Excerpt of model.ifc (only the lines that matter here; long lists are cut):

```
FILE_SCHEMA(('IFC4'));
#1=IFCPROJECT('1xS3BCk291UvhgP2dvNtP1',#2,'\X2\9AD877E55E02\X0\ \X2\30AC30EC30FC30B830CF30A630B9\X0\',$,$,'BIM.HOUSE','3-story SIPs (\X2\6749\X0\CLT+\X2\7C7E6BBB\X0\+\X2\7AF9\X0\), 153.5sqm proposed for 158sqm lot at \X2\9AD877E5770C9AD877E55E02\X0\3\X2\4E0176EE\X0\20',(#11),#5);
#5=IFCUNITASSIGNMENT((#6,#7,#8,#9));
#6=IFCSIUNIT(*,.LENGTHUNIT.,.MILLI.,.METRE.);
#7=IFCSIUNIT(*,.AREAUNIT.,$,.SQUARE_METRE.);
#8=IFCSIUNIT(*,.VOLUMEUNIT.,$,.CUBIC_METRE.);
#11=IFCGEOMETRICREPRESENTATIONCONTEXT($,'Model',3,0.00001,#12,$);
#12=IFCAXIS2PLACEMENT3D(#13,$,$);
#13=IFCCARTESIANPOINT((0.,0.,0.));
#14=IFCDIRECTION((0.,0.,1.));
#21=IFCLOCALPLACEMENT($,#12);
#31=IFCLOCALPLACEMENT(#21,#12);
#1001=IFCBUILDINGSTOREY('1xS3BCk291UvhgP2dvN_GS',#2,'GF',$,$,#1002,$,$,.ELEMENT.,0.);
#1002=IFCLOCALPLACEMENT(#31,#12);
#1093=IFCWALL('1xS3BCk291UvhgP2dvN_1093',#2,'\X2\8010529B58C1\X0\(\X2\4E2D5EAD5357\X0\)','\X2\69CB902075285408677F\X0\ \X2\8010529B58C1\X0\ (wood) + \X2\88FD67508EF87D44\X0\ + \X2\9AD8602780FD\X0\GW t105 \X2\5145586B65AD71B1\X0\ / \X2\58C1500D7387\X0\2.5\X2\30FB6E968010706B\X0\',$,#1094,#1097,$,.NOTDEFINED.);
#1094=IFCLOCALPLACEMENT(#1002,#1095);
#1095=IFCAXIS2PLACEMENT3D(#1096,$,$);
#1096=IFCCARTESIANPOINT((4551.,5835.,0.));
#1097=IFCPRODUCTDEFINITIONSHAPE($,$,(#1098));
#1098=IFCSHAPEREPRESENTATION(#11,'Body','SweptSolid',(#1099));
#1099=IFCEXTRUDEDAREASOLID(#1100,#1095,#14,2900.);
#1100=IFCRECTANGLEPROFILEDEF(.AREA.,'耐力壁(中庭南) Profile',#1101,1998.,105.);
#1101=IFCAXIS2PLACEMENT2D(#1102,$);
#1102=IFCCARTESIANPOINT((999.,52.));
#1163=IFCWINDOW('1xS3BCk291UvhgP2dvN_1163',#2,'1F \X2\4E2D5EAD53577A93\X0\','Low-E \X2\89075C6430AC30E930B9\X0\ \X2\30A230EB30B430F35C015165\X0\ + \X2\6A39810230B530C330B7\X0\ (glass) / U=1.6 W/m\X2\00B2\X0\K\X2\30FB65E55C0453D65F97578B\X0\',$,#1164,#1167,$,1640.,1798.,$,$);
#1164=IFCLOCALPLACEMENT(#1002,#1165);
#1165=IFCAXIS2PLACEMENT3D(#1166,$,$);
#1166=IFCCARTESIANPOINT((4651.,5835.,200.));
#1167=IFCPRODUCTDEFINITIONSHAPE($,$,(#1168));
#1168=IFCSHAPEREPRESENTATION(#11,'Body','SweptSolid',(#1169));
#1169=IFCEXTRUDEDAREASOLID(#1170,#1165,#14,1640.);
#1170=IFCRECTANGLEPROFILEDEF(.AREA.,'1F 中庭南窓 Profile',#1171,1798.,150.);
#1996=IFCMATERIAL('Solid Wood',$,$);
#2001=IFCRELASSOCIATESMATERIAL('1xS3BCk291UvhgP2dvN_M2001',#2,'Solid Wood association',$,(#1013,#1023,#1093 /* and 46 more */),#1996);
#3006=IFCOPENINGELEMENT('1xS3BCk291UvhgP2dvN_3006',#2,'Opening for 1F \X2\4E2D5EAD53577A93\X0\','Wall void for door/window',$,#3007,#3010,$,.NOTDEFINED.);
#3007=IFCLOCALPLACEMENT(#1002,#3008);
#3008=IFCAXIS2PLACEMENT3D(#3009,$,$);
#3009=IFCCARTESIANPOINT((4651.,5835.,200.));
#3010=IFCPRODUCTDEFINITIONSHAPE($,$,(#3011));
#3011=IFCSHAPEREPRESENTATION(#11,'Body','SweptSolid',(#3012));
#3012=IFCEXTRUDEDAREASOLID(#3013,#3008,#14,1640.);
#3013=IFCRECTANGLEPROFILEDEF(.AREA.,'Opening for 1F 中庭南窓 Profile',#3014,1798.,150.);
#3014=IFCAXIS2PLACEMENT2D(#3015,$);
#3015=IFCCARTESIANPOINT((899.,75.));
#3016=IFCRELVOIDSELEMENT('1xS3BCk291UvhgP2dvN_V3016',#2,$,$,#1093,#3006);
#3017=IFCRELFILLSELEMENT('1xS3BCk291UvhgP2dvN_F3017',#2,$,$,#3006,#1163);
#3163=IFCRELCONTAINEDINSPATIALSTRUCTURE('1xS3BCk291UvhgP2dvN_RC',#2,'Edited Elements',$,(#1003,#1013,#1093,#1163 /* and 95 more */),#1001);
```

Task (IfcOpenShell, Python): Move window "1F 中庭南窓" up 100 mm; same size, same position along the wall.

```python
import numpy as np
import ifcopenshell
import ifcopenshell.api.geometry
import ifcopenshell.util.placement
import ifcopenshell.util.unit

model = ifcopenshell.open("model.ifc")
unit_scale = ifcopenshell.util.unit.calculate_unit_scale(model)

window = model.by_id(1163)
opening = window.FillsVoids[0].RelatingOpeningElement
dz = 0.1 / unit_scale

shift = np.array([0.0, 0.0, dz])
# The window is not placed relative to its opening, so move both.
for product in (opening, window):
    matrix = ifcopenshell.util.placement.get_local_placement(product.ObjectPlacement)
    matrix[:3, 3] += shift
    ifcopenshell.api.geometry.edit_object_placement(model, product=product, matrix=matrix, is_si=False)

print(f"moved by {dz * unit_scale:+.3f} m")

model.write("model_v2.ifc")
```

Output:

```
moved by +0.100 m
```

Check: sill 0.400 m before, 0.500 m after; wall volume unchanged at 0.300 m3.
